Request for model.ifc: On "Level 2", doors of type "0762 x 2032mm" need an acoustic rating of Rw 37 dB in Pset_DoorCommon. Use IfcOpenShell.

First a look at what the model holds.

```python
import ifcopenshell
import ifcopenshell.util.element

model = ifcopenshell.open("model.ifc")
print(model.schema)
storey = next(s for s in model.by_type("IfcBuildingStorey") if s.Name == "Level 2")
doors = [e for e in ifcopenshell.util.element.get_decomposition(storey) if e.is_a("IfcDoor")]
seen = {}
for e in doors:
    element_type = ifcopenshell.util.element.get_type(e)
    key = (element_type.Name if element_type != e and element_type else None, ifcopenshell.util.element.get_pset(e, "Pset_DoorCommon", "AcousticRating"))
    seen[key] = seen.get(key, 0) + 1
for (name, value), count in sorted(seen.items(), key=str):
    print(count, "x", name, "|", value)
```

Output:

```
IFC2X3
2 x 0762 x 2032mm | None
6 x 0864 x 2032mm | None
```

```python
import ifcopenshell
import ifcopenshell.api.pset
import ifcopenshell.util.element

model = ifcopenshell.open("model.ifc")

storey = next(s for s in model.by_type("IfcBuildingStorey") if s.Name == "Level 2")
doors = [e for e in ifcopenshell.util.element.get_decomposition(storey) if e.is_a("IfcDoor")]

count = 0
for e in doors:
    element_type = ifcopenshell.util.element.get_type(e)
    if element_type in (None, e) or element_type.Name != "0762 x 2032mm":
        continue
    # add_pset returns the element's existing set when there is one.
    pset = ifcopenshell.api.pset.add_pset(model, product=e, name="Pset_DoorCommon")
    ifcopenshell.api.pset.edit_pset(model, pset=pset, properties={"AcousticRating": "Rw 37 dB"})
    count += 1

print(count, "doors updated")

model.write("model_updated.ifc")
```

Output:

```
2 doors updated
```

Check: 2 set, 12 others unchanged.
